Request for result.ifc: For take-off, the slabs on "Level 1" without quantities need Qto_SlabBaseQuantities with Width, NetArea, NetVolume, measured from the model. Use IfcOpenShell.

First a look at what the model holds.

```python
import ifcopenshell
import ifcopenshell.util.element
import ifcopenshell.util.unit

model = ifcopenshell.open("result.ifc")
print(model.schema)
for unit_type in ("LENGTHUNIT", "AREAUNIT", "VOLUMEUNIT"):
    print(unit_type, ifcopenshell.util.unit.calculate_unit_scale(model, unit_type))
storey = next(s for s in model.by_type("IfcBuildingStorey") if s.Name == "Level 1")
slabs = [e for e in ifcopenshell.util.element.get_decomposition(storey) if e.is_a("IfcSlab")]
for e in sorted(slabs, key=lambda e: e.id()):
    print(e.id(), e.is_a(), e.Name, list(ifcopenshell.util.element.get_psets(e, qtos_only=True)), sep=" | ")
```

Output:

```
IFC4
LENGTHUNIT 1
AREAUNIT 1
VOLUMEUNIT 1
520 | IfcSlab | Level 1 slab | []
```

```python
import ifcopenshell
import ifcopenshell.api.pset
import ifcopenshell.geom
import ifcopenshell.util.element
import ifcopenshell.util.shape
import ifcopenshell.util.unit

model = ifcopenshell.open("result.ifc")
unit_scale = ifcopenshell.util.unit.calculate_unit_scale(model)
area_scale = ifcopenshell.util.unit.calculate_unit_scale(model, "AREAUNIT")
volume_scale = ifcopenshell.util.unit.calculate_unit_scale(model, "VOLUMEUNIT")
settings = ifcopenshell.geom.settings()

storey = next(s for s in model.by_type("IfcBuildingStorey") if s.Name == "Level 1")
slabs = [e for e in ifcopenshell.util.element.get_decomposition(storey) if e.is_a("IfcSlab")]

for e in sorted(slabs, key=lambda e: e.id()):
    if ifcopenshell.util.element.get_psets(e, qtos_only=True, should_inherit=False):
        continue
    # Geometry comes back in metres, in the element's own axes.
    shape = ifcopenshell.geom.create_shape(settings, e)
    values = {
        "Width": ifcopenshell.util.shape.get_z(shape.geometry) / unit_scale,
        "NetArea": ifcopenshell.util.shape.get_footprint_area(shape.geometry) / area_scale,
        "NetVolume": ifcopenshell.util.shape.get_volume(shape.geometry) / volume_scale,
    }
    qto = ifcopenshell.api.pset.add_qto(model, product=e, name="Qto_SlabBaseQuantities")
    ifcopenshell.api.pset.edit_qto(model, qto=qto, properties=values)
    print(e.id(), {k: round(v, 3) for k, v in values.items()})

model.write("result_updated.ifc")
```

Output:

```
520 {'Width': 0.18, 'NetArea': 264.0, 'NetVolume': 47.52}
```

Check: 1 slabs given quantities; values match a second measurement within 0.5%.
